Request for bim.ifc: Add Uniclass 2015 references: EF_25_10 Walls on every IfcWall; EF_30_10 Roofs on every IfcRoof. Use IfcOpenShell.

First a look at what the model holds.

```python
import ifcopenshell

model = ifcopenshell.open("bim.ifc")
print(model.schema)
print("classifications:", [c.Name for c in model.by_type("IfcClassification")])
for ifc_class in ("IfcDoor", "IfcRoof", "IfcStair", "IfcWall", "IfcWindow"):
    print(ifc_class, len(model.by_type(ifc_class)))
```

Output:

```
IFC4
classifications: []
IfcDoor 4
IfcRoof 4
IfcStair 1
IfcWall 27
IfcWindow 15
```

```python
import ifcopenshell
import ifcopenshell.api.classification

model = ifcopenshell.open("bim.ifc")

system = ifcopenshell.api.classification.add_classification(model, classification="Uniclass 2015")

codes = {
    "IfcWall": ("EF_25_10", "Walls"),
    "IfcRoof": ("EF_30_10", "Roofs"),
}
for ifc_class, (code, name) in codes.items():
    products = model.by_type(ifc_class)
    ifcopenshell.api.classification.add_reference(
        model, products=products, classification=system, identification=code, name=name
    )
    print(code, len(products))

model.write("bim-out.ifc")
```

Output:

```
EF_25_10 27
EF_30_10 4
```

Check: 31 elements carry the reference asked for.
